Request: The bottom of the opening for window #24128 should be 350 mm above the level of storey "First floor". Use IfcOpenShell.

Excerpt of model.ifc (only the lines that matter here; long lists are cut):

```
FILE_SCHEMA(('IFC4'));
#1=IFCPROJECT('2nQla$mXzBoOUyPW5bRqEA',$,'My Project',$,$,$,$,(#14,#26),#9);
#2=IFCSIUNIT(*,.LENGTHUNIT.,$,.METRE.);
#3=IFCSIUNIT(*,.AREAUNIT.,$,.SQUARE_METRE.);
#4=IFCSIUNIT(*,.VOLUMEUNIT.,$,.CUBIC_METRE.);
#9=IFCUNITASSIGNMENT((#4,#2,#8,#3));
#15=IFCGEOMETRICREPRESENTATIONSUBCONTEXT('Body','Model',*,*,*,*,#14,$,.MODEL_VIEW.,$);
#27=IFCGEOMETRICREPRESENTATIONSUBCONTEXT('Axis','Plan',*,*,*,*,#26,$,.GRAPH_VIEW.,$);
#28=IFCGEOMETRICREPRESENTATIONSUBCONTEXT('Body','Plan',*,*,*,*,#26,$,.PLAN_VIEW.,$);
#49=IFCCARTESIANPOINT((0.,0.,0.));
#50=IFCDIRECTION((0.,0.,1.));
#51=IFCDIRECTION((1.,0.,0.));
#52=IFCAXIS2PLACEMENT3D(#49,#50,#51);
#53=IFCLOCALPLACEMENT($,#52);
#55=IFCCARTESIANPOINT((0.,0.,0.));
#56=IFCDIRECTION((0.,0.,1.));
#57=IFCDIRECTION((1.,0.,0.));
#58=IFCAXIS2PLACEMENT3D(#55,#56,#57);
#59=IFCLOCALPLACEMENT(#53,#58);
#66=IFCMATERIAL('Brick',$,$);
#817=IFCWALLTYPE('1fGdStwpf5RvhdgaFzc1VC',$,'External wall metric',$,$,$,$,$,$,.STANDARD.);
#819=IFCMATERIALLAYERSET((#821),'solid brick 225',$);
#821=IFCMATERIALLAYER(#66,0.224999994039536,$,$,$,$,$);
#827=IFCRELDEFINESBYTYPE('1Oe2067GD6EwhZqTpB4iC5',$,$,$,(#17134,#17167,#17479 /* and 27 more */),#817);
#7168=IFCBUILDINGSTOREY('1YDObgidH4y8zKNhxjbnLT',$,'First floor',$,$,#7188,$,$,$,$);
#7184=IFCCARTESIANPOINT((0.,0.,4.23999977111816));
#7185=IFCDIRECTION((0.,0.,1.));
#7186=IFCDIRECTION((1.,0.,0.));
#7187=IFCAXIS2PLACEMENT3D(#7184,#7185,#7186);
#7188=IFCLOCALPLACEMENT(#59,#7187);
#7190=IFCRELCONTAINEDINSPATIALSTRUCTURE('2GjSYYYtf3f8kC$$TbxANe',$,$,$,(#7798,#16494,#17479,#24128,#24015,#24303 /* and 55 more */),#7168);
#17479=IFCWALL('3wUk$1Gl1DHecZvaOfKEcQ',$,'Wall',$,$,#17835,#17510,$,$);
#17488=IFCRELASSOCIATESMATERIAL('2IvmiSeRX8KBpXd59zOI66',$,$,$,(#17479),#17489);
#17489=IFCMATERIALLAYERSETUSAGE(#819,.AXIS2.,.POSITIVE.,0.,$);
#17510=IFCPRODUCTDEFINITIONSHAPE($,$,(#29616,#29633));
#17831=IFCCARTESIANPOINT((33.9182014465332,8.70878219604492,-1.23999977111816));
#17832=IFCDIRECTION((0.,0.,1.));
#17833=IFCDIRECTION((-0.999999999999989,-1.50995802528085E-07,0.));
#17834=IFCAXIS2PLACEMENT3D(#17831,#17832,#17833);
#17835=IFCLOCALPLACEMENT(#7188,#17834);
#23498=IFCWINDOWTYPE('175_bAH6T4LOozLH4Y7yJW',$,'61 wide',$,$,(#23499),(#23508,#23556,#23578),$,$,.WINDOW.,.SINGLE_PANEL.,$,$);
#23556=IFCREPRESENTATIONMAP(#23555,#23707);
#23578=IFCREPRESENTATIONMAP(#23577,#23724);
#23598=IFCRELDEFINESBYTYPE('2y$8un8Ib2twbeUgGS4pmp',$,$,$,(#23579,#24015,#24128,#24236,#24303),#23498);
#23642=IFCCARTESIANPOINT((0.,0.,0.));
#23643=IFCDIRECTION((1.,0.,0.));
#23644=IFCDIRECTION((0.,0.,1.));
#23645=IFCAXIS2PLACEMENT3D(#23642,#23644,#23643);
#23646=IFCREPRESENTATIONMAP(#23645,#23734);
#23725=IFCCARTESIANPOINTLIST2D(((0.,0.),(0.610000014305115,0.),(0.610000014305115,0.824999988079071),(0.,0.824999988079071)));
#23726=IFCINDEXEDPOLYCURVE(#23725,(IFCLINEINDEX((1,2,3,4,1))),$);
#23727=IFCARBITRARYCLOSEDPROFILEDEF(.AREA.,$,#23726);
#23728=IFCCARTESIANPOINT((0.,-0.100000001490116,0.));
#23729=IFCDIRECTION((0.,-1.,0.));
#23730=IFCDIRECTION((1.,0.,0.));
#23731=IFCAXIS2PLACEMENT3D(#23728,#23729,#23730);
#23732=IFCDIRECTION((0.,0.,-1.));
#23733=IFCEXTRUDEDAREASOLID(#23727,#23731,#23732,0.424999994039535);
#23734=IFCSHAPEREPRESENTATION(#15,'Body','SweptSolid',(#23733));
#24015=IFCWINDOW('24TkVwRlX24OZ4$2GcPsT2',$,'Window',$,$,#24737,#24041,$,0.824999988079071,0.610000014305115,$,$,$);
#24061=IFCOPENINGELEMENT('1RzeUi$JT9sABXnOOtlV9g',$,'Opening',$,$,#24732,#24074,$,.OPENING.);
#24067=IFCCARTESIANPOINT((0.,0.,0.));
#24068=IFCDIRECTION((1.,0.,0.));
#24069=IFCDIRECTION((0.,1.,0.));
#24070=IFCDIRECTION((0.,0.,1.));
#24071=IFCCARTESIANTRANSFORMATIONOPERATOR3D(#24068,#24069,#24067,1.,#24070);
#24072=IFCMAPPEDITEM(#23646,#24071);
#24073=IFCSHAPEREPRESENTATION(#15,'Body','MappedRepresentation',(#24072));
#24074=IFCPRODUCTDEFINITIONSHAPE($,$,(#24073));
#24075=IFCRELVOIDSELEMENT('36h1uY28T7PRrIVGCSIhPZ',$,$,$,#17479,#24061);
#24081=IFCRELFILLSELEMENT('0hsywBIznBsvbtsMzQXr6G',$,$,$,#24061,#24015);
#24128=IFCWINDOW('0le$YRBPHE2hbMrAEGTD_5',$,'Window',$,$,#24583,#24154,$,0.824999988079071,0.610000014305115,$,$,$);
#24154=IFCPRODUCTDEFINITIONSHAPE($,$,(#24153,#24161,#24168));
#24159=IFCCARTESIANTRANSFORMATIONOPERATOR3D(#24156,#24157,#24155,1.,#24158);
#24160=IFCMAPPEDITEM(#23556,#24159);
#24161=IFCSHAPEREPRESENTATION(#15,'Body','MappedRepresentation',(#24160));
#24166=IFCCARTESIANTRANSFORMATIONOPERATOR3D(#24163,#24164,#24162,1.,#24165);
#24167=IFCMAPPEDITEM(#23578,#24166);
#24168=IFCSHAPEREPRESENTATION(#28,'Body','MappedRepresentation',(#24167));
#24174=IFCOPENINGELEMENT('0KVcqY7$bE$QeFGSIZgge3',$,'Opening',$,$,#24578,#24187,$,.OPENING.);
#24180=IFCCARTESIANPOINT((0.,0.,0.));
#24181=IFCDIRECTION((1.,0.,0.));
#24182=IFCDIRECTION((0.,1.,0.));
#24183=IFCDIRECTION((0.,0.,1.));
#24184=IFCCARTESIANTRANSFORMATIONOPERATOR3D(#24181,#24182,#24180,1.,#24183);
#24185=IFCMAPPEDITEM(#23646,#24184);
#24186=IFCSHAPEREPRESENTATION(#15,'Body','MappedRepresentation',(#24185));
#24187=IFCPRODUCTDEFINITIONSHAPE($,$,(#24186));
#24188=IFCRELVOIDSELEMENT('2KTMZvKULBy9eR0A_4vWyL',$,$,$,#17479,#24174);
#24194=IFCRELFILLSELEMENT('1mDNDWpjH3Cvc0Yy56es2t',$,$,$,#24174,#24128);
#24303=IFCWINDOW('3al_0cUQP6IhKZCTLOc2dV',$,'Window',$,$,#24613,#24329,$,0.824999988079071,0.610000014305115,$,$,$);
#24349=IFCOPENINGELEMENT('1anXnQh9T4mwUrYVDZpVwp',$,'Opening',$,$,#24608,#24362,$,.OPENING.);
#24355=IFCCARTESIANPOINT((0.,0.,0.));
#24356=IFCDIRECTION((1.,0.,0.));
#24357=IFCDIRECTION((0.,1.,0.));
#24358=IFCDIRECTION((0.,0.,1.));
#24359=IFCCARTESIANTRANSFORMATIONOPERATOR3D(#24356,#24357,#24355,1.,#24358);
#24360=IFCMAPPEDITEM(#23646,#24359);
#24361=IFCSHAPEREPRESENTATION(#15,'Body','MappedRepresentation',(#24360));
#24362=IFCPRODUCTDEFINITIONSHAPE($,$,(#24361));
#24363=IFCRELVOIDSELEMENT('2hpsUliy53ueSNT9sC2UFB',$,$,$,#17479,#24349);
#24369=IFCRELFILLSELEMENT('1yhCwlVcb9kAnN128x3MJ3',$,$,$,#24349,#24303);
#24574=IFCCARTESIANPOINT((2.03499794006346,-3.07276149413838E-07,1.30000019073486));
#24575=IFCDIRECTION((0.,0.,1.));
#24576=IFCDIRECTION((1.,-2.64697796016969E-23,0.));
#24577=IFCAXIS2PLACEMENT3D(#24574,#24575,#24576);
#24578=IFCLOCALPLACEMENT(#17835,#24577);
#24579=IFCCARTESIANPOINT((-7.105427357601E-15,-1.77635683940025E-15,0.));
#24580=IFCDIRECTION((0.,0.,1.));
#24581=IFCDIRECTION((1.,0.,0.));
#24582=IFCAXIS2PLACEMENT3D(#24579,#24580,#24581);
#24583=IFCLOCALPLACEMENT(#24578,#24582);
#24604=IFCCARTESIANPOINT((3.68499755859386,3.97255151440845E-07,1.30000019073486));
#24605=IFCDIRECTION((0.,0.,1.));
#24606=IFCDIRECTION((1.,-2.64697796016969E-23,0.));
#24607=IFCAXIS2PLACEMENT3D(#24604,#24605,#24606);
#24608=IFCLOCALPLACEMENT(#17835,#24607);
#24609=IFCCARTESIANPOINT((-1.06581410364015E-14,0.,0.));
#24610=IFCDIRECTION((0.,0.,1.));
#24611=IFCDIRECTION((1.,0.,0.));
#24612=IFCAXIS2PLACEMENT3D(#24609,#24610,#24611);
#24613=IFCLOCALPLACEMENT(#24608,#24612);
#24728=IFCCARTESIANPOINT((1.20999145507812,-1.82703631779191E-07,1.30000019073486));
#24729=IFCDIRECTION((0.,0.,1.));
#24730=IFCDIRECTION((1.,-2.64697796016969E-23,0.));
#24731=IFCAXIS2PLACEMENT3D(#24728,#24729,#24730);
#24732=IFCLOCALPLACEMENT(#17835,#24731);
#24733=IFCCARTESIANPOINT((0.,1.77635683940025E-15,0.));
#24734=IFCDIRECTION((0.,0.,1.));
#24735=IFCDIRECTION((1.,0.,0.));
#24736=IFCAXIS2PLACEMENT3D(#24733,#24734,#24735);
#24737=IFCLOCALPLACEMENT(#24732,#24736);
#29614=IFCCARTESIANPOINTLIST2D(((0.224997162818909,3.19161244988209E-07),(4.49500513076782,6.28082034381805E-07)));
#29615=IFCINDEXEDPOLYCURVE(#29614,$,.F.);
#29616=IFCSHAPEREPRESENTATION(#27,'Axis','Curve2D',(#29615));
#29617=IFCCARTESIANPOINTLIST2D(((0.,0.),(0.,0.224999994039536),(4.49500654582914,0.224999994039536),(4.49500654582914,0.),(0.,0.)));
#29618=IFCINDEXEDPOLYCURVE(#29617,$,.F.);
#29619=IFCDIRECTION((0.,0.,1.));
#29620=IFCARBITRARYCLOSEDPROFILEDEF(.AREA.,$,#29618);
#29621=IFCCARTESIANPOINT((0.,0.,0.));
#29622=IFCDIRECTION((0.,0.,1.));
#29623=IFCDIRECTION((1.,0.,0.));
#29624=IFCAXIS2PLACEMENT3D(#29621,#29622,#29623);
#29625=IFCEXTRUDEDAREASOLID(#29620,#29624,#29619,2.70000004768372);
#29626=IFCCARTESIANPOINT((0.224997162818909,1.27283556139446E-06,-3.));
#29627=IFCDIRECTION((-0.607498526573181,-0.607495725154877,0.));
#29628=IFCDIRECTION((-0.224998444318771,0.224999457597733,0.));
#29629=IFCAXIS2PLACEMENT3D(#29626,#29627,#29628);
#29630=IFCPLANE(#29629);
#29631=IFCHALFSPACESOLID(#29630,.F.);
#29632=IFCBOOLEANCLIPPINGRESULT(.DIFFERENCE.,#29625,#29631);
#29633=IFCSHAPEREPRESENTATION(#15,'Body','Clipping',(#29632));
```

```python
import numpy as np
import ifcopenshell
import ifcopenshell.api.geometry
import ifcopenshell.geom
import ifcopenshell.util.element
import ifcopenshell.util.placement
import ifcopenshell.util.shape
import ifcopenshell.util.unit

model = ifcopenshell.open("model.ifc")
unit_scale = ifcopenshell.util.unit.calculate_unit_scale(model)

window = model.by_id(24128)
opening = window.FillsVoids[0].RelatingOpeningElement
storey = ifcopenshell.util.element.get_container(window, ifc_class="IfcBuildingStorey")
level = ifcopenshell.util.placement.get_local_placement(storey.ObjectPlacement)[2, 3]

# The opening's origin need not be at the sill, so measure its lowest point.
shape = ifcopenshell.geom.create_shape(ifcopenshell.geom.settings(), opening)
bottom = ifcopenshell.util.shape.get_shape_bottom_elevation(shape, shape.geometry) / unit_scale
dz = level + 0.35 / unit_scale - bottom

shift = np.array([0.0, 0.0, dz])
# The window is placed relative to its opening, so it follows when the opening moves.
matrix = ifcopenshell.util.placement.get_local_placement(opening.ObjectPlacement)
matrix[:3, 3] += shift
ifcopenshell.api.geometry.edit_object_placement(
    model, product=opening, matrix=matrix, is_si=False, should_transform_children=True
)

print(f"moved by {dz * unit_scale:+.3f} m")

model.write("model_v2.ifc")
```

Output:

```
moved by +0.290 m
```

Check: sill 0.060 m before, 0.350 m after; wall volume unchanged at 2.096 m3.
